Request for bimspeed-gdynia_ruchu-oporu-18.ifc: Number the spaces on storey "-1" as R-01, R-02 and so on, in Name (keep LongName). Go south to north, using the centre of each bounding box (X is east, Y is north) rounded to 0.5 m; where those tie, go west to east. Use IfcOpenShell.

First a look at what the model holds.

```python
import ifcopenshell
import ifcopenshell.util.element
import ifcopenshell.util.placement

model = ifcopenshell.open("bimspeed-gdynia_ruchu-oporu-18.ifc")
print(model.schema)
storey = next(s for s in model.by_type("IfcBuildingStorey") if s.Name == "-1")
spaces = [e for e in ifcopenshell.util.element.get_decomposition(storey) if e.is_a("IfcSpace")]
for e in sorted(spaces, key=lambda e: e.id()):
    origin = ifcopenshell.util.placement.get_local_placement(e.ObjectPlacement)[:3, 3]
    print(e.id(), e.Name, e.LongName, origin.round(2) + 0.0, sep=" | ")
```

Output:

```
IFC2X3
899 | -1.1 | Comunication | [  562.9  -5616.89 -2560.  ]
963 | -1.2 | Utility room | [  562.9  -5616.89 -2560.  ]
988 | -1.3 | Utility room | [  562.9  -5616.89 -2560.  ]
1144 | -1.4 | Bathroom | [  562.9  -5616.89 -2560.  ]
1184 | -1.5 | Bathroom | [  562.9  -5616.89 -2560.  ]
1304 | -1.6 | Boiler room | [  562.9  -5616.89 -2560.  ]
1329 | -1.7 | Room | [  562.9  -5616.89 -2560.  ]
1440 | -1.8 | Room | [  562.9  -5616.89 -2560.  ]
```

```python
import ifcopenshell
import ifcopenshell.geom
import ifcopenshell.util.element
import ifcopenshell.util.shape

model = ifcopenshell.open("bimspeed-gdynia_ruchu-oporu-18.ifc")
settings = ifcopenshell.geom.settings()
settings.set("use-world-coords", True)


def centre(element):
    shape = ifcopenshell.geom.create_shape(settings, element)
    return ifcopenshell.util.shape.get_bbox_centroid(shape.geometry)


storey = next(s for s in model.by_type("IfcBuildingStorey") if s.Name == "-1")
spaces = [e for e in ifcopenshell.util.element.get_decomposition(storey) if e.is_a("IfcSpace")]

# Insertion points can sit at a corner or the storey origin, so sort by the geometry (in metres).
centres = {e: centre(e) for e in spaces}
spaces.sort(key=lambda e: (round(centres[e][1] / 0.5), centres[e][0]))

for i, e in enumerate(spaces, start=1):
    number = f"R-{i:02d}"
    e.Name = number
    print(e.id(), number)

model.write("bimspeed-gdynia_ruchu-oporu-18-out.ifc")
```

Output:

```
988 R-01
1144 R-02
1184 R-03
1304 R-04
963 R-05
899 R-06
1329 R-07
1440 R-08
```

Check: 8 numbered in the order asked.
